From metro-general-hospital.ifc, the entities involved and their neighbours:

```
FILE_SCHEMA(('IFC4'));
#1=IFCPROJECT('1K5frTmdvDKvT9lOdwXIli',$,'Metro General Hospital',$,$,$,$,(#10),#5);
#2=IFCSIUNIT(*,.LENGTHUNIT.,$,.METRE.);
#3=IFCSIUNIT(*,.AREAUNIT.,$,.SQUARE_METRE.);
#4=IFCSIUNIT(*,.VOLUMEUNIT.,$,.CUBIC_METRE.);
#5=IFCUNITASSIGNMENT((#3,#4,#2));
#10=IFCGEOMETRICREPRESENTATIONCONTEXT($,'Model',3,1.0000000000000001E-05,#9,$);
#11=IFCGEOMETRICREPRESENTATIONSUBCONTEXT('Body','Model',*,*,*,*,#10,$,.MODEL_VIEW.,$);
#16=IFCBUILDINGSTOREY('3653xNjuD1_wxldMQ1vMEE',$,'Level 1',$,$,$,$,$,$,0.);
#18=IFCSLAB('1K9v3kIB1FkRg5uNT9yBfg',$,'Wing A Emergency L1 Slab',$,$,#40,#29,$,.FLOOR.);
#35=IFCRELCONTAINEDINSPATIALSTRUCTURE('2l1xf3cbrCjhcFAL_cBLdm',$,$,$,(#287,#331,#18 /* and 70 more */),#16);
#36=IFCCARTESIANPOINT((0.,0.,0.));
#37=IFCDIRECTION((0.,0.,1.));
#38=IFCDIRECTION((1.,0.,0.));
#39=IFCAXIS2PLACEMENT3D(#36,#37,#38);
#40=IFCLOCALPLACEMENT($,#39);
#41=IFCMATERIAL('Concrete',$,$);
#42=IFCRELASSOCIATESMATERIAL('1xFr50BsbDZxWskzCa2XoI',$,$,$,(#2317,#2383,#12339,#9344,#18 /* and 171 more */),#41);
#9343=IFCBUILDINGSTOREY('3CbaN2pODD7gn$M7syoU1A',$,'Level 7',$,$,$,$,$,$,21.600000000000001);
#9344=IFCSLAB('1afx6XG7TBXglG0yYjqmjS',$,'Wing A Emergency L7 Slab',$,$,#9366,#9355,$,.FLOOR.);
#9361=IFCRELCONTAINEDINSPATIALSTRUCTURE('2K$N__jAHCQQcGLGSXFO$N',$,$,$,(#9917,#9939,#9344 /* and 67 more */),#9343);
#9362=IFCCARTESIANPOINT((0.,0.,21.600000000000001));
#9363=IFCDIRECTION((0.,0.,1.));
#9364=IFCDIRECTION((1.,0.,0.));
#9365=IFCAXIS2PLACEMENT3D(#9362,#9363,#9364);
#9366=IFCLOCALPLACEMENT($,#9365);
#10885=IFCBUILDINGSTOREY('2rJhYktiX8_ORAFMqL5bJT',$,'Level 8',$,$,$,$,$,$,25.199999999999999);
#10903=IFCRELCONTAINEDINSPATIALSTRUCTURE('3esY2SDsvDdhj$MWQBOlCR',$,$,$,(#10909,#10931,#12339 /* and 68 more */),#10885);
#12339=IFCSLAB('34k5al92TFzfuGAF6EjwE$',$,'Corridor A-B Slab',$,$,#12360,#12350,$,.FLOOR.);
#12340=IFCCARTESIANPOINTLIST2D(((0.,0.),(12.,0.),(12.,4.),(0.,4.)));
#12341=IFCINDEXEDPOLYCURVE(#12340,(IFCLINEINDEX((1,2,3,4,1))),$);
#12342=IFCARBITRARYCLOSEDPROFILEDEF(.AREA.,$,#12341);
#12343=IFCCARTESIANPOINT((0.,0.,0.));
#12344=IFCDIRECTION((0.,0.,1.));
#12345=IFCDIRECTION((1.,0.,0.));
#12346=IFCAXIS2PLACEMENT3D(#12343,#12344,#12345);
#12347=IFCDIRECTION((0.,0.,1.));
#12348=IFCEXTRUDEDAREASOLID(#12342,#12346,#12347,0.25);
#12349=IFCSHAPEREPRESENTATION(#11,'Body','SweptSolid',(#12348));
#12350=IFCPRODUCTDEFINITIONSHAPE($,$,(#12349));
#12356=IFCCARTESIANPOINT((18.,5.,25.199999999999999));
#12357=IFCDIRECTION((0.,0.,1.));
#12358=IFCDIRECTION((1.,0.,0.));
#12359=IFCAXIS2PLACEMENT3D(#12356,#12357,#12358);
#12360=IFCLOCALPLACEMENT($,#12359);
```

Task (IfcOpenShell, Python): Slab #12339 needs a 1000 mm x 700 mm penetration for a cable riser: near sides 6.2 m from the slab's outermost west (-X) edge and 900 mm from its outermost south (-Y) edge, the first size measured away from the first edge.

```python
import numpy as np
import ifcopenshell
import ifcopenshell.api.feature
import ifcopenshell.api.geometry
import ifcopenshell.api.root
import ifcopenshell.geom
import ifcopenshell.util.placement
import ifcopenshell.util.representation
import ifcopenshell.util.shape
import ifcopenshell.util.unit

model = ifcopenshell.open("metro-general-hospital.ifc")
unit_scale = ifcopenshell.util.unit.calculate_unit_scale(model)
settings = ifcopenshell.geom.settings()


def volume(element):
    """Net volume in cubic metres, openings subtracted."""
    shape = ifcopenshell.geom.create_shape(settings, element)
    return ifcopenshell.util.shape.get_volume(shape.geometry)


slab = model.by_guid("34k5al92TFzfuGAF6EjwE$")
before = volume(slab)

# Extent in the slab's own axes, in metres. The edges named are its -X and -Y sides.
slab_shape = ifcopenshell.geom.create_shape(settings, slab)
vertices = ifcopenshell.util.shape.get_vertices(slab_shape.geometry)
x_min, y_min, bottom = vertices.min(axis=0)
top = vertices[:, 2].max()

opening = ifcopenshell.api.root.create_entity(model, ifc_class="IfcOpeningElement", name="Cable riser opening", predefined_type="OPENING")
context = ifcopenshell.util.representation.get_context(model, "Model", "Body", "MODEL_VIEW")
width, depth = 1, 0.7
outline = [(0.0, 0.0), (width, 0.0), (width, depth), (0.0, depth), (0.0, 0.0)]
# Overshoot both faces by 50 mm so the cut is clean.
shape = ifcopenshell.api.geometry.add_slab_representation(
    model, context=context, depth=top - bottom + 0.1, polyline=outline
)
ifcopenshell.api.geometry.assign_representation(model, product=opening, representation=shape)

matrix = ifcopenshell.util.placement.get_local_placement(slab.ObjectPlacement)
matrix[:, 3] = matrix @ np.append(np.array([x_min + 6.2, y_min + 0.9, bottom - 0.05]) / unit_scale, 1.0)
ifcopenshell.api.geometry.edit_object_placement(model, product=opening, matrix=matrix, is_si=False)
ifcopenshell.api.feature.add_feature(model, feature=opening, element=slab)

after = volume(slab)

print(f"slab volume {before:.3f} -> {after:.3f} m3")

model.write("metro-general-hospital_edited.ifc")
```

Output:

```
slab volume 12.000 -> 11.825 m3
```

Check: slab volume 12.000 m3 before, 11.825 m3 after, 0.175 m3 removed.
